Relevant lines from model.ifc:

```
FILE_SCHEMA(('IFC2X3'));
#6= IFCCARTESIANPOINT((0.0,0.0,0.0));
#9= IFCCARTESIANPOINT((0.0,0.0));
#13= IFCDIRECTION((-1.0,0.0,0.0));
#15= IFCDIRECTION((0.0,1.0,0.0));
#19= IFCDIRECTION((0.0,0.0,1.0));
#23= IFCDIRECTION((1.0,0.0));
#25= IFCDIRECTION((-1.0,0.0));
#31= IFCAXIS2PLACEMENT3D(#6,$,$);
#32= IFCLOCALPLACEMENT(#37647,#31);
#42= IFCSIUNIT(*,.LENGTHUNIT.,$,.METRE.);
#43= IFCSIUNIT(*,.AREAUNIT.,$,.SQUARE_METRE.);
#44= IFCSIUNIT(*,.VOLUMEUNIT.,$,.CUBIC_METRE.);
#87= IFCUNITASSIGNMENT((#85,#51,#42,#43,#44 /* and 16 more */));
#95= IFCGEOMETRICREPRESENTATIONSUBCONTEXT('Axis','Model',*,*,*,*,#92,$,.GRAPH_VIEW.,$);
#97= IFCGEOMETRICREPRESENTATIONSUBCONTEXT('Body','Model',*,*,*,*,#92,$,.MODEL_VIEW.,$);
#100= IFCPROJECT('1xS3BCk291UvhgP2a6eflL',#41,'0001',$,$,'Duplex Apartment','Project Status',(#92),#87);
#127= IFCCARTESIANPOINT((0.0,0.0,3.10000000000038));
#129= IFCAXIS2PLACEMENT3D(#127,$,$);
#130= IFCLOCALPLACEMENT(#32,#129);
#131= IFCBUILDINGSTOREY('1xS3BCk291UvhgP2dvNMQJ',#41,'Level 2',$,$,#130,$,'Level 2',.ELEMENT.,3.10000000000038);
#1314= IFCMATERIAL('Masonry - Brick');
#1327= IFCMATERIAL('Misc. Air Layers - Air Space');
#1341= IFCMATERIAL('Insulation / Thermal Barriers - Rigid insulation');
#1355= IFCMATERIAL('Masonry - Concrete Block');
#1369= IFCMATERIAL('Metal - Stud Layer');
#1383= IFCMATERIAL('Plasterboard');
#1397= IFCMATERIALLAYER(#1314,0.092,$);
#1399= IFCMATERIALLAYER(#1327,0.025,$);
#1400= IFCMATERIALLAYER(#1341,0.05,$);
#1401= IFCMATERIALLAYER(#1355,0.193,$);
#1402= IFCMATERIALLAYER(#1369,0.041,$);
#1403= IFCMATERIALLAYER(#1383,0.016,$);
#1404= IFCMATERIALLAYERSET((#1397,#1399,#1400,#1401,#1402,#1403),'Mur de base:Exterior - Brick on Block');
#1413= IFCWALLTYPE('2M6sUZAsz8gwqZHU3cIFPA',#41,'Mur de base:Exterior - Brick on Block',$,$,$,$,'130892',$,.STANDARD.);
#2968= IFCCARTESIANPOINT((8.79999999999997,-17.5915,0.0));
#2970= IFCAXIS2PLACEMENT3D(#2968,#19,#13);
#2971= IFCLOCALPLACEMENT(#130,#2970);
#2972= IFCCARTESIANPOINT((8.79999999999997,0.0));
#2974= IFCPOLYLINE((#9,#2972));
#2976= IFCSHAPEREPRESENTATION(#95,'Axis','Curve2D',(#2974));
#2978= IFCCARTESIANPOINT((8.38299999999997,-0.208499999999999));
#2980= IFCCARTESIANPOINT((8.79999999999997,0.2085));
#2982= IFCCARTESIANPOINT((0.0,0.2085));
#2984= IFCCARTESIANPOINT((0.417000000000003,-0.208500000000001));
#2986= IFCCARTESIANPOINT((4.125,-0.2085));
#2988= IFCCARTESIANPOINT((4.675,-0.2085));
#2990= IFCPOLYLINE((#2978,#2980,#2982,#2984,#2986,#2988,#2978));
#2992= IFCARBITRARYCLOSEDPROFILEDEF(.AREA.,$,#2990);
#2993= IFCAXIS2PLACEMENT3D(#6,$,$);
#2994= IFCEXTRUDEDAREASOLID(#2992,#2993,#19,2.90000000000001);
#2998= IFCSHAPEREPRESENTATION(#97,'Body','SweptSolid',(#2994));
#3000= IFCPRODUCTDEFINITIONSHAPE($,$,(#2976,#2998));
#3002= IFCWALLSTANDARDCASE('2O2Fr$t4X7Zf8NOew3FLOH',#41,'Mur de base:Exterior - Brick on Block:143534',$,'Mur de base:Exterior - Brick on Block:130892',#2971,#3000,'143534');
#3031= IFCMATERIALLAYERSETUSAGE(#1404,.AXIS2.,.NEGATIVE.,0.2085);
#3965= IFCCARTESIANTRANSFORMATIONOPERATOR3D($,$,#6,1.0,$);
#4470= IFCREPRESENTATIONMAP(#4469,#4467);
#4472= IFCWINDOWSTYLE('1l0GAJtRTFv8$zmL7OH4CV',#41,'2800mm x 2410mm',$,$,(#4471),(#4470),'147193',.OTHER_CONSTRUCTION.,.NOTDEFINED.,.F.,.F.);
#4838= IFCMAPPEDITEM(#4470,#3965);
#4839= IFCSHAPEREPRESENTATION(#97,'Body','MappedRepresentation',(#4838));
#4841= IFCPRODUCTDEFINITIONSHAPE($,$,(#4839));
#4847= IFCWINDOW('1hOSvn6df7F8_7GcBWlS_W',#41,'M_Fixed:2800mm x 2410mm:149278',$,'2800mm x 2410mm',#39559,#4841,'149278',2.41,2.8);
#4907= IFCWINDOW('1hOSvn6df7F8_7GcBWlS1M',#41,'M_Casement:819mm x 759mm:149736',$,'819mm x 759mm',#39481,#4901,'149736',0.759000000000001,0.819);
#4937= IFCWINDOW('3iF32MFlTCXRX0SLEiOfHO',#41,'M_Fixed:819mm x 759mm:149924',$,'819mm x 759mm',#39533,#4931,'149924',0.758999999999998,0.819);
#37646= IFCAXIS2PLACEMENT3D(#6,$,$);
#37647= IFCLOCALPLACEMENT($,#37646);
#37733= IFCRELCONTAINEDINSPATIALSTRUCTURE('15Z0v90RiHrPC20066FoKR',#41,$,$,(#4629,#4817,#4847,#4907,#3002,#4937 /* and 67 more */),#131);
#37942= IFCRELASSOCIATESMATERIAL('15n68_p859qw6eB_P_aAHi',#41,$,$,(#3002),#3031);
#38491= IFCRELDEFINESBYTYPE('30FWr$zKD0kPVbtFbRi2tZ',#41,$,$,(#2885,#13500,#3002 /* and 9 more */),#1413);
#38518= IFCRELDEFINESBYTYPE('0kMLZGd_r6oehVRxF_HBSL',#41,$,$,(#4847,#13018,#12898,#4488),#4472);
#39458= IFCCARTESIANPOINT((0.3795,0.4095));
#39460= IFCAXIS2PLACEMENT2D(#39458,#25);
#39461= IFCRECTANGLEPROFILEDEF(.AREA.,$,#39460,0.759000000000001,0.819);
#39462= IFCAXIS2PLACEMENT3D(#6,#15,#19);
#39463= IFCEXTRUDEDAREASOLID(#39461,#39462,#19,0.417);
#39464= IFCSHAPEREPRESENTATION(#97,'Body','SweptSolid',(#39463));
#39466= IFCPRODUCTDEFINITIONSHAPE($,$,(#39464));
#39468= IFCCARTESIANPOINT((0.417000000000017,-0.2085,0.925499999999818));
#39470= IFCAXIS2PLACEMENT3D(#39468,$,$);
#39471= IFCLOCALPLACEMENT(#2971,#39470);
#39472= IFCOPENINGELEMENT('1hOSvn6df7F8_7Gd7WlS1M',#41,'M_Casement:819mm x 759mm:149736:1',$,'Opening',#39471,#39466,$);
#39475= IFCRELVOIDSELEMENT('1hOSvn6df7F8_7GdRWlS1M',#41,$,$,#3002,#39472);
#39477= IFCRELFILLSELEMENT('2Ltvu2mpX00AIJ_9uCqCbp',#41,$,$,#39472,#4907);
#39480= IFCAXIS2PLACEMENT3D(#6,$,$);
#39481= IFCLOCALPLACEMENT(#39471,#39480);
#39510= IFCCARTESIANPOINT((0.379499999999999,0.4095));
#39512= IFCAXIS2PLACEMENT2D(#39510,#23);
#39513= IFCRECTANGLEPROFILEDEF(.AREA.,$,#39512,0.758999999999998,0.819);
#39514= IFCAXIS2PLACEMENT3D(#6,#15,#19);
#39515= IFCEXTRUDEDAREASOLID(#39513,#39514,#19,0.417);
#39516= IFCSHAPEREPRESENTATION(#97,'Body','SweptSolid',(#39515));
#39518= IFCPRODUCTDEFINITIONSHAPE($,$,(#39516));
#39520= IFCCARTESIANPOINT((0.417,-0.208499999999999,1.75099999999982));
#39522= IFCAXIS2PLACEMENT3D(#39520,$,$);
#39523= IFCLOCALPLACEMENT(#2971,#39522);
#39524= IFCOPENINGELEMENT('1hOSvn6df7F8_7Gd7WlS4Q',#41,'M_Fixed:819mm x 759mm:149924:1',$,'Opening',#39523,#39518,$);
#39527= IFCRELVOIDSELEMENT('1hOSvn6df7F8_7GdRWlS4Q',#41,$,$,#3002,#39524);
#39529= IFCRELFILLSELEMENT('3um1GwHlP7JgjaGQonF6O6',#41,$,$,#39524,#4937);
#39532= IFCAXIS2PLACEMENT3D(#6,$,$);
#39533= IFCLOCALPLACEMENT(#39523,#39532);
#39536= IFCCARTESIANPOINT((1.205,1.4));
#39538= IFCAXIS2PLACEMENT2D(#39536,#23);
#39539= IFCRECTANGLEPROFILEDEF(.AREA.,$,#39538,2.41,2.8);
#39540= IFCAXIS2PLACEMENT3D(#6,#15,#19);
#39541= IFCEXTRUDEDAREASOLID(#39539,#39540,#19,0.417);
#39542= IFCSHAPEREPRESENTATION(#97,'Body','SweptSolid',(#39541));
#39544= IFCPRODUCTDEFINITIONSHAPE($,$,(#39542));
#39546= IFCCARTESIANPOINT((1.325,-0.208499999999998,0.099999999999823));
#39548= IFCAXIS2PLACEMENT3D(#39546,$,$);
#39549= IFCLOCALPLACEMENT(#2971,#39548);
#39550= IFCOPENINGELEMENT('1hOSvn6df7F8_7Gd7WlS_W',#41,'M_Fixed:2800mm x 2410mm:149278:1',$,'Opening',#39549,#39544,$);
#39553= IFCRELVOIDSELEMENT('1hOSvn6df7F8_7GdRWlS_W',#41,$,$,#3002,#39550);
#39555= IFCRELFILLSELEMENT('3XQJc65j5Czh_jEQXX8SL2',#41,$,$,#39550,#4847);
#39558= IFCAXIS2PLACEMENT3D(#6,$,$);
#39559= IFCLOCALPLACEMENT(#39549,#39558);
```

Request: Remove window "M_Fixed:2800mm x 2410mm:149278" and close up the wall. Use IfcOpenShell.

```python
import ifcopenshell
import ifcopenshell.api.feature
import ifcopenshell.api.root
import ifcopenshell.geom
import ifcopenshell.util.shape

model = ifcopenshell.open("model.ifc")
settings = ifcopenshell.geom.settings()


def volume(element):
    """Net volume in cubic metres, openings subtracted."""
    shape = ifcopenshell.geom.create_shape(settings, element)
    return ifcopenshell.util.shape.get_volume(shape.geometry)


window = model.by_guid("1hOSvn6df7F8_7GcBWlS_W")
opening = window.FillsVoids[0].RelatingOpeningElement
wall = opening.VoidsElements[0].RelatingBuildingElement
before = volume(wall)

ifcopenshell.api.root.remove_product(model, product=window)
ifcopenshell.api.feature.remove_feature(model, feature=opening)

after = volume(wall)

print(f"wall volume {before:.3f} -> {after:.3f} m3")

model.write("model_updated.ifc")
```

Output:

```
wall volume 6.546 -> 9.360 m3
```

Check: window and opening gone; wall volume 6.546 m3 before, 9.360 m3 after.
